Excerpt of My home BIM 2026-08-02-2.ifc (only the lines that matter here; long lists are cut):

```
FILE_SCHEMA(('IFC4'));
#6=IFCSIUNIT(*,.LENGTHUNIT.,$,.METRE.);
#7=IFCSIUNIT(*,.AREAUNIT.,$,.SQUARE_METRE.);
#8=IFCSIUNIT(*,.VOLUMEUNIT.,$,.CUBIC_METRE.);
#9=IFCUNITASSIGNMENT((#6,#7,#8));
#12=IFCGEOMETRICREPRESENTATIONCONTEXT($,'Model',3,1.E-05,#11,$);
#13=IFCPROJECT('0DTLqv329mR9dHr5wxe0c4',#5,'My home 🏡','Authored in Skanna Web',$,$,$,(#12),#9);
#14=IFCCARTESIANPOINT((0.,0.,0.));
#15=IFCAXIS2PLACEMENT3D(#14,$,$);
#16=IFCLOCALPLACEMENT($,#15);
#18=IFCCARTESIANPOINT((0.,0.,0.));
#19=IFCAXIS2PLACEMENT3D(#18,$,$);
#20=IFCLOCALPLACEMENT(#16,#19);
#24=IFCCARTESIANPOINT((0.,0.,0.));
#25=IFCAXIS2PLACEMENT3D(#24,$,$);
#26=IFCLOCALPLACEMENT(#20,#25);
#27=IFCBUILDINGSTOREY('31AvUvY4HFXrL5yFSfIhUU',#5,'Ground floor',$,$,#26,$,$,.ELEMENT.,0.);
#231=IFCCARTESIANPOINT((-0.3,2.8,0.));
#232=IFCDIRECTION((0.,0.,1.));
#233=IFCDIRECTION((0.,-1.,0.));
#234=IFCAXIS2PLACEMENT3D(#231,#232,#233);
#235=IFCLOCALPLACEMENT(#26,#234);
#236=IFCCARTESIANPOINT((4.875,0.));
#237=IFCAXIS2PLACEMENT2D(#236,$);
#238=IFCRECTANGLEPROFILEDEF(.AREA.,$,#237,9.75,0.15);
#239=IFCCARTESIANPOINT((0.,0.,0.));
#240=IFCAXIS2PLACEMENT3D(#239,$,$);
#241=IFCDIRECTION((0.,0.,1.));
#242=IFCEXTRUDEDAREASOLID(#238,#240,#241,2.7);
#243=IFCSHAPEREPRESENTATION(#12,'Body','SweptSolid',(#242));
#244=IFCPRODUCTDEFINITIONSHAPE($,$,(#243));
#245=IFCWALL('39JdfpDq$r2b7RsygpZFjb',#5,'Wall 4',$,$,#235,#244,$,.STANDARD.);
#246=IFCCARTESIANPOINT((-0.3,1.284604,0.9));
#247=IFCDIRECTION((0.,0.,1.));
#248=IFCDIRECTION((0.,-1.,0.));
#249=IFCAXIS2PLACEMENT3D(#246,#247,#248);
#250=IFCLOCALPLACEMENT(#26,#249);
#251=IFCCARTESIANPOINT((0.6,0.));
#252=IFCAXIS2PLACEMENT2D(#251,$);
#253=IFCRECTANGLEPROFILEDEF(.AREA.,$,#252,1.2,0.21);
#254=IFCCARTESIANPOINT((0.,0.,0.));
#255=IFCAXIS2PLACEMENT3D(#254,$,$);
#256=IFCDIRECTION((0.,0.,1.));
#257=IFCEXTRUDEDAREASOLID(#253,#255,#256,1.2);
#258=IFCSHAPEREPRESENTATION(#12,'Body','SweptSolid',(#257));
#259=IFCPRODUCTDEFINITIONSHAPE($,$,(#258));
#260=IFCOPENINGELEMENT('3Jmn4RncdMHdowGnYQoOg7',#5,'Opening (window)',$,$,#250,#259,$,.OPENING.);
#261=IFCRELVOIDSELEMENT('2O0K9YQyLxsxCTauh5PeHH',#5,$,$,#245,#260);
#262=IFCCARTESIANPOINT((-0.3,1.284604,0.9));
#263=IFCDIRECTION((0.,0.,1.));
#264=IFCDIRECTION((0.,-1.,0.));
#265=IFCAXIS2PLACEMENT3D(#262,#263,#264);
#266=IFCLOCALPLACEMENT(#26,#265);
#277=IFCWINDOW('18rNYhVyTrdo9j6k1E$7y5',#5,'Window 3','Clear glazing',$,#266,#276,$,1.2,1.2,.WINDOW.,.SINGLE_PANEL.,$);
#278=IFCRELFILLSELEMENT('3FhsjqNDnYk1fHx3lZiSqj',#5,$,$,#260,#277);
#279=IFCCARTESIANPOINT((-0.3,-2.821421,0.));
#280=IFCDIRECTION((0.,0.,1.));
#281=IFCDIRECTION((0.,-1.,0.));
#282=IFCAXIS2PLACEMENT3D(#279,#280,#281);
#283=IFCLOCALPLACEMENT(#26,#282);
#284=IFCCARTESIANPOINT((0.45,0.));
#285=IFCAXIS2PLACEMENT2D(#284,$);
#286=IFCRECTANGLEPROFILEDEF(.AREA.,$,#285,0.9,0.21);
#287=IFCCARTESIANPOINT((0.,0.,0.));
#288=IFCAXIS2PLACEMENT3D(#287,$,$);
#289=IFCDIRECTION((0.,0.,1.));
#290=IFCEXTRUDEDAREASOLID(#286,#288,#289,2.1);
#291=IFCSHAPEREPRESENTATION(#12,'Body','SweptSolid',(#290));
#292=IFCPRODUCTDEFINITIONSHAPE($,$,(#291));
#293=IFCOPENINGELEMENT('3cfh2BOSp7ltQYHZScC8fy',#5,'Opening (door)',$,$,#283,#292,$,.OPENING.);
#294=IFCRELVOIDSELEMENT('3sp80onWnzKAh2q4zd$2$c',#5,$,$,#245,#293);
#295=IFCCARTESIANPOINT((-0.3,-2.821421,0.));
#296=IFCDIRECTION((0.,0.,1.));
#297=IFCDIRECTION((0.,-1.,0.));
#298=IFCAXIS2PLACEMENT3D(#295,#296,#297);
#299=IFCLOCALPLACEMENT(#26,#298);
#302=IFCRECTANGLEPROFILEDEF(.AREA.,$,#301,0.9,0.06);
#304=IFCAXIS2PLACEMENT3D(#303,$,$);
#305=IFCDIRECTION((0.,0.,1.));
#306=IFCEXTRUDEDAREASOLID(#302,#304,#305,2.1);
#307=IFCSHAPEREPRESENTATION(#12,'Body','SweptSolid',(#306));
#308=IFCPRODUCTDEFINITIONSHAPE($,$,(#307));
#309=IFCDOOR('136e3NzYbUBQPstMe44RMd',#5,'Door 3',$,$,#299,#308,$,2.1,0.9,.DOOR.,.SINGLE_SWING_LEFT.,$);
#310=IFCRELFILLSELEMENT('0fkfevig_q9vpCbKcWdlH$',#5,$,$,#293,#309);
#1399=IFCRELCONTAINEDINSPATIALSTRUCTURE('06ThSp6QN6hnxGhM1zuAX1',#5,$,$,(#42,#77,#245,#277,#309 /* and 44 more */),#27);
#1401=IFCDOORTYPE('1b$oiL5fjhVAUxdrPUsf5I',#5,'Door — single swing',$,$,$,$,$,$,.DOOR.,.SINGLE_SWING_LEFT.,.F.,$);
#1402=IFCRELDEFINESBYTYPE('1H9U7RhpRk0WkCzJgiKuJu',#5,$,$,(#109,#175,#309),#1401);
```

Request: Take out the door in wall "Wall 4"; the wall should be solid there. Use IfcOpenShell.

```python
import ifcopenshell
import ifcopenshell.api.feature
import ifcopenshell.api.root
import ifcopenshell.geom
import ifcopenshell.util.shape

model = ifcopenshell.open("My home BIM 2026-08-02-2.ifc")
settings = ifcopenshell.geom.settings()


def volume(element):
    """Net volume in cubic metres, openings subtracted."""
    shape = ifcopenshell.geom.create_shape(settings, element)
    return ifcopenshell.util.shape.get_volume(shape.geometry)


door = model.by_id(309)
opening = door.FillsVoids[0].RelatingOpeningElement
wall = opening.VoidsElements[0].RelatingBuildingElement
before = volume(wall)

ifcopenshell.api.root.remove_product(model, product=door)
ifcopenshell.api.feature.remove_feature(model, feature=opening)

after = volume(wall)

print(f"wall volume {before:.3f} -> {after:.3f} m3")

model.write("My home BIM 2026-08-02-2_edited.ifc")
```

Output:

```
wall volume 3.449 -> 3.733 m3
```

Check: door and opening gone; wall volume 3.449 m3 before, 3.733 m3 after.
